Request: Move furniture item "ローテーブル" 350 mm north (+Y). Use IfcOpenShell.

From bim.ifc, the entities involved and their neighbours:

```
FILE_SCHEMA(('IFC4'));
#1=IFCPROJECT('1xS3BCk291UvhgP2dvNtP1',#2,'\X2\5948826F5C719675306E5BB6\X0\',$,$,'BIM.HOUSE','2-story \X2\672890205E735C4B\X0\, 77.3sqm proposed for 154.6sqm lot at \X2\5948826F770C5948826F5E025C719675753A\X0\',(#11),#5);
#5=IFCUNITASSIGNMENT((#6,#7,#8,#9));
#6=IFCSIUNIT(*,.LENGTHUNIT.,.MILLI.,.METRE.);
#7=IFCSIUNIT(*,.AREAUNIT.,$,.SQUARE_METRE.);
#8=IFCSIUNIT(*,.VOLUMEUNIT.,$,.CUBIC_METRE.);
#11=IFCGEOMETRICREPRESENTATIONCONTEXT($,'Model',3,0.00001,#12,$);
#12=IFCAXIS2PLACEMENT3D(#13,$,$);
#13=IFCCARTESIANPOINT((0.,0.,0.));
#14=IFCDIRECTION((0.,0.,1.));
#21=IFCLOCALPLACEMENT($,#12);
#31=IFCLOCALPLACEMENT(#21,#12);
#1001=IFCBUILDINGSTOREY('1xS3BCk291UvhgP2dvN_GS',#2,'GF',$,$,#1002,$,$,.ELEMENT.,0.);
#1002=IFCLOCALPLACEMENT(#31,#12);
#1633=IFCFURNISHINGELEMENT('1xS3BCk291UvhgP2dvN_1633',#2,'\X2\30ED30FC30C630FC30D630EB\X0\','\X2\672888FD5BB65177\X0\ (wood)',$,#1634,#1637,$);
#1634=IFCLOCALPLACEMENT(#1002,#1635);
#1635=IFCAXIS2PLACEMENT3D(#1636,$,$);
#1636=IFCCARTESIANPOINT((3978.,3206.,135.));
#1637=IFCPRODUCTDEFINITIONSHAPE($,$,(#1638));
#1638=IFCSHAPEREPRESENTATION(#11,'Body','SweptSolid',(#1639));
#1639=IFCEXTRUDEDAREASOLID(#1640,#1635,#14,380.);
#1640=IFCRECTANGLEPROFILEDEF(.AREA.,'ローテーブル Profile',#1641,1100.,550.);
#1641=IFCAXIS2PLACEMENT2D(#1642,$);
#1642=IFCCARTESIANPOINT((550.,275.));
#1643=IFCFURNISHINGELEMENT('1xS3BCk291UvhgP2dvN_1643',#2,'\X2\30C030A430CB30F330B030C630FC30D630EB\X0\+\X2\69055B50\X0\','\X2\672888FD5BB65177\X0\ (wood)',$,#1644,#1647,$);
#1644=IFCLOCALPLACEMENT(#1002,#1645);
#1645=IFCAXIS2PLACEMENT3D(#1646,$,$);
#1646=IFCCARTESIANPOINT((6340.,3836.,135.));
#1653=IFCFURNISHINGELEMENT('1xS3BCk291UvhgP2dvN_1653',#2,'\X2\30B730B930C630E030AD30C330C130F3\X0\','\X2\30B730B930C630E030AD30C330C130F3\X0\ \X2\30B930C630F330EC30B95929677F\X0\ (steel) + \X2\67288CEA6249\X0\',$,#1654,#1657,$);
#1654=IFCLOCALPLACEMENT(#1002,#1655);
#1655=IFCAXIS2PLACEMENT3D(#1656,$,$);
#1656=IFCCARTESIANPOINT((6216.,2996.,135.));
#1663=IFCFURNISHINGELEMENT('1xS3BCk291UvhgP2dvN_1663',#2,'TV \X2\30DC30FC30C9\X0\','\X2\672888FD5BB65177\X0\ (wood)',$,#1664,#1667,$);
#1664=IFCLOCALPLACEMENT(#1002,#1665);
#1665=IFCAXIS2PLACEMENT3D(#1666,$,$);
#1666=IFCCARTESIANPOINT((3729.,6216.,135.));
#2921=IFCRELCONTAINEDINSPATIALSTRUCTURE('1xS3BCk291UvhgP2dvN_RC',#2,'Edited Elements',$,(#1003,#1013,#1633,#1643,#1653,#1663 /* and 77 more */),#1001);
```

```python
import ifcopenshell
import ifcopenshell.api.geometry
import ifcopenshell.util.placement
import ifcopenshell.util.unit

model = ifcopenshell.open("bim.ifc")
unit_scale = ifcopenshell.util.unit.calculate_unit_scale(model)

item = model.by_guid("1xS3BCk291UvhgP2dvN_1633")
matrix = ifcopenshell.util.placement.get_local_placement(item.ObjectPlacement)
matrix[1, 3] += 0.35 / unit_scale
ifcopenshell.api.geometry.edit_object_placement(model, product=item, matrix=matrix, is_si=False)

print(ifcopenshell.util.placement.get_local_placement(item.ObjectPlacement).round(3) + 0.0)

model.write("bim_edited.ifc")
```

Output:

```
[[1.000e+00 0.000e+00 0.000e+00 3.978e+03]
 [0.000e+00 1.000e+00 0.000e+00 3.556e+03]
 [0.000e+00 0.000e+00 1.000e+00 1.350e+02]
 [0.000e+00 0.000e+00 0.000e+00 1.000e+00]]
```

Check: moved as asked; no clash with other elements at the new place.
